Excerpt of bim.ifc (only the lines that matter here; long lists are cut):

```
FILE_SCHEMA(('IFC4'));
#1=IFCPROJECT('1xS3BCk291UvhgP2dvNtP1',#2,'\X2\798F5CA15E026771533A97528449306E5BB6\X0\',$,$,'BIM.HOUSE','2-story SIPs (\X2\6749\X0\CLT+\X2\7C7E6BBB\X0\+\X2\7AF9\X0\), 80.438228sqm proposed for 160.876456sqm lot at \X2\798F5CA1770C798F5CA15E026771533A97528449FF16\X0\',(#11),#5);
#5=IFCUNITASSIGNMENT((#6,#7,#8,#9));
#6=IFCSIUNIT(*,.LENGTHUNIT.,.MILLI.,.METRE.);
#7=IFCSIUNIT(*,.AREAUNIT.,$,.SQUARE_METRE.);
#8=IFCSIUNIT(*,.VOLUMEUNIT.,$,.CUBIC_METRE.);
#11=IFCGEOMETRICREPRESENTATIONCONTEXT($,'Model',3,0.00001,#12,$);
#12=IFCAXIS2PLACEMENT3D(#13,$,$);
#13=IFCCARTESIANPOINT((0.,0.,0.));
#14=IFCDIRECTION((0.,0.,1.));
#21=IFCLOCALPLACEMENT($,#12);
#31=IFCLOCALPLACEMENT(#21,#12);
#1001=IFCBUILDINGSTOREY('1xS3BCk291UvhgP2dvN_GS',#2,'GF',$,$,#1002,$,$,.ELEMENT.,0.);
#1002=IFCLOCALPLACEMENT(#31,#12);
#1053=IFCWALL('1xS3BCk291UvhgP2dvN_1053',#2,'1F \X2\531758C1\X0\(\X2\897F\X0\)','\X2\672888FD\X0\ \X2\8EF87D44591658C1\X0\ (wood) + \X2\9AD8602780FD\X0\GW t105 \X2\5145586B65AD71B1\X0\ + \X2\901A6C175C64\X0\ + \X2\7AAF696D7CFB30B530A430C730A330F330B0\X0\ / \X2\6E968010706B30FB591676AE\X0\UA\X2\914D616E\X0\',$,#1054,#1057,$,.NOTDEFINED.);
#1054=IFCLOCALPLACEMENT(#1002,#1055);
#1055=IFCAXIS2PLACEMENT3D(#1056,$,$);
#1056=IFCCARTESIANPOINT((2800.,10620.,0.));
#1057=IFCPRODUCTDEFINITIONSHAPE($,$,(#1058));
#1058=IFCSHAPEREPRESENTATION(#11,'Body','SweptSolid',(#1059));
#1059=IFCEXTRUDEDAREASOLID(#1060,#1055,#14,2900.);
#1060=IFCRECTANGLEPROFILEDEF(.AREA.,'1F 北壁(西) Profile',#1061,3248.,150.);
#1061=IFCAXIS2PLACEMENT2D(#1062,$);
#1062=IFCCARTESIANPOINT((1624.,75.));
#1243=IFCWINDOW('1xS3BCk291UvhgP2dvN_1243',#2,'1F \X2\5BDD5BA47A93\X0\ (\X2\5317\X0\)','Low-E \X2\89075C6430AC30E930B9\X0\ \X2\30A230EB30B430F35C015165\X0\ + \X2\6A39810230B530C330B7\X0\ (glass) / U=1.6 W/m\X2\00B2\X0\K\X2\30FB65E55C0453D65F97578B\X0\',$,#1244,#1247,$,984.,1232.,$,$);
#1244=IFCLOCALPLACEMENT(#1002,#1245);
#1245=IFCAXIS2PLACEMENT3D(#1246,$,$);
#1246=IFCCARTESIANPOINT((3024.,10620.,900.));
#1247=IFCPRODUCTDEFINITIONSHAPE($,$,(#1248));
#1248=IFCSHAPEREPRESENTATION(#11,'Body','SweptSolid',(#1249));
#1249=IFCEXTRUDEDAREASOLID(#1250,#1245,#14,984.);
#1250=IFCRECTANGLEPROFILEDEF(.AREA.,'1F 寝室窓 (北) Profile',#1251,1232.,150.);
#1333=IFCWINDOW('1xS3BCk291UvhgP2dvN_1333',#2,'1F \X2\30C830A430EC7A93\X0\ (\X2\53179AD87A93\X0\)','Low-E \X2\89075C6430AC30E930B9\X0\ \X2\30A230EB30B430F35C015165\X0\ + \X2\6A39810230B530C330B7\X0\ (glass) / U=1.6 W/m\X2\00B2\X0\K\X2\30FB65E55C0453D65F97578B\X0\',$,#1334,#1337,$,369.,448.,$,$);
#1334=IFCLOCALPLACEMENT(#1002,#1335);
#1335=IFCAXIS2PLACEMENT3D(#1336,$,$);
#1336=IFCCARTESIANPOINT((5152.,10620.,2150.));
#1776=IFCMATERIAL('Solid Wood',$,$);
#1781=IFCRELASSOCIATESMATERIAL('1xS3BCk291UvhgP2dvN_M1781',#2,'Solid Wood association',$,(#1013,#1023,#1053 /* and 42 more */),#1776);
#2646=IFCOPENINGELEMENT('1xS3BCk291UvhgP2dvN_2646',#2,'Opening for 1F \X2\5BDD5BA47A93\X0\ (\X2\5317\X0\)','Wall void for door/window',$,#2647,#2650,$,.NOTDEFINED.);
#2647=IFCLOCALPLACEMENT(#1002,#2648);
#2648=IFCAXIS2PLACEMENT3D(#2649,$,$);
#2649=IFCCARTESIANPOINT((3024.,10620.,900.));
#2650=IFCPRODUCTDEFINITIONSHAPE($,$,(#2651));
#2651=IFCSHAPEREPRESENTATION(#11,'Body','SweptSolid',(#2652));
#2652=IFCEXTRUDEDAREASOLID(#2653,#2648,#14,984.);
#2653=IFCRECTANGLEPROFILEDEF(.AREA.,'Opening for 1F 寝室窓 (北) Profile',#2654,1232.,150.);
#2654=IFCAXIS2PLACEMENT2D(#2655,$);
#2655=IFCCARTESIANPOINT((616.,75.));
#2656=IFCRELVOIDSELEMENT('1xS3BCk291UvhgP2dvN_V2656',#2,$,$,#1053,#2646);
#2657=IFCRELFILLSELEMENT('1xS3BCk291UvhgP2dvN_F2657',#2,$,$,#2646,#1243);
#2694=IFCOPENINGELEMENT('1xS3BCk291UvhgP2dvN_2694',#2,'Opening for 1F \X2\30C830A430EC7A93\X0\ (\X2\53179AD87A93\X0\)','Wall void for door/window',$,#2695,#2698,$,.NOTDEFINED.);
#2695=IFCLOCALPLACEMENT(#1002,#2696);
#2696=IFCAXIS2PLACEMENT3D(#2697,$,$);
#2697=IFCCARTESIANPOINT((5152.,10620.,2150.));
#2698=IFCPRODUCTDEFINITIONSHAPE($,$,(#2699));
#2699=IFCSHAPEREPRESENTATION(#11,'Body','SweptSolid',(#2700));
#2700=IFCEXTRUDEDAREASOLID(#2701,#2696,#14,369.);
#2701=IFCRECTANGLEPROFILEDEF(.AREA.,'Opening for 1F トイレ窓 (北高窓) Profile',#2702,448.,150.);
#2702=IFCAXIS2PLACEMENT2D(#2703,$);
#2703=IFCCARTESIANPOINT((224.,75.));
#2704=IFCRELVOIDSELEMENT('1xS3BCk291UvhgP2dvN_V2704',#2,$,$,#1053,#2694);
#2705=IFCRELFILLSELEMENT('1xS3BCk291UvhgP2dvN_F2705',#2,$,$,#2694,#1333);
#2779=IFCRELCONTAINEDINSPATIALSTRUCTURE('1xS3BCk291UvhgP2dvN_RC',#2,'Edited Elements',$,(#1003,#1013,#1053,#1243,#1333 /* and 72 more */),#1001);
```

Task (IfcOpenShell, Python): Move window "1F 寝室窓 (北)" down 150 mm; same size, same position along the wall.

```python
import numpy as np
import ifcopenshell
import ifcopenshell.api.geometry
import ifcopenshell.util.placement
import ifcopenshell.util.unit

model = ifcopenshell.open("bim.ifc")
unit_scale = ifcopenshell.util.unit.calculate_unit_scale(model)

window = model.by_guid("1xS3BCk291UvhgP2dvN_1243")
opening = window.FillsVoids[0].RelatingOpeningElement
dz = -150.0

shift = np.array([0.0, 0.0, dz])
# The window is not placed relative to its opening, so move both.
for product in (opening, window):
    matrix = ifcopenshell.util.placement.get_local_placement(product.ObjectPlacement)
    matrix[:3, 3] += shift
    ifcopenshell.api.geometry.edit_object_placement(model, product=product, matrix=matrix, is_si=False)

print(f"moved by {dz * unit_scale:+.3f} m")

model.write("bim-out.ifc")
```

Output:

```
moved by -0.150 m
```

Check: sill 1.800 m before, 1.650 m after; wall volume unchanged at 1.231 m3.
